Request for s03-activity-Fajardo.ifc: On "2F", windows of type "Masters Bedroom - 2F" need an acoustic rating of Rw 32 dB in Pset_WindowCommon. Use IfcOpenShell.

First a look at what the model holds.

```python
import ifcopenshell
import ifcopenshell.util.element

model = ifcopenshell.open("s03-activity-Fajardo.ifc")
print(model.schema)
storey = next(s for s in model.by_type("IfcBuildingStorey") if s.Name == "2F")
windows = [e for e in ifcopenshell.util.element.get_decomposition(storey) if e.is_a("IfcWindow")]
seen = {}
for e in windows:
    element_type = ifcopenshell.util.element.get_type(e)
    key = (element_type.Name if element_type != e and element_type else None, ifcopenshell.util.element.get_pset(e, "Pset_WindowCommon", "AcousticRating"))
    seen[key] = seen.get(key, 0) + 1
for (name, value), count in sorted(seen.items(), key=str):
    print(count, "x", name, "|", value)
```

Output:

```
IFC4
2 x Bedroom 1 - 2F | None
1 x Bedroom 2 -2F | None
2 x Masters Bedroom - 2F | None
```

```python
import ifcopenshell
import ifcopenshell.api.pset
import ifcopenshell.util.element

model = ifcopenshell.open("s03-activity-Fajardo.ifc")

storey = next(s for s in model.by_type("IfcBuildingStorey") if s.Name == "2F")
windows = [e for e in ifcopenshell.util.element.get_decomposition(storey) if e.is_a("IfcWindow")]

count = 0
for e in windows:
    element_type = ifcopenshell.util.element.get_type(e)
    if element_type in (None, e) or element_type.Name != "Masters Bedroom - 2F":
        continue
    # add_pset returns the element's existing set when there is one.
    pset = ifcopenshell.api.pset.add_pset(model, product=e, name="Pset_WindowCommon")
    ifcopenshell.api.pset.edit_pset(model, pset=pset, properties={"AcousticRating": "Rw 32 dB"})
    count += 1

print(count, "windows updated")

model.write("s03-activity-Fajardo-out.ifc")
```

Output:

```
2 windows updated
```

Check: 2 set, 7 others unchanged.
